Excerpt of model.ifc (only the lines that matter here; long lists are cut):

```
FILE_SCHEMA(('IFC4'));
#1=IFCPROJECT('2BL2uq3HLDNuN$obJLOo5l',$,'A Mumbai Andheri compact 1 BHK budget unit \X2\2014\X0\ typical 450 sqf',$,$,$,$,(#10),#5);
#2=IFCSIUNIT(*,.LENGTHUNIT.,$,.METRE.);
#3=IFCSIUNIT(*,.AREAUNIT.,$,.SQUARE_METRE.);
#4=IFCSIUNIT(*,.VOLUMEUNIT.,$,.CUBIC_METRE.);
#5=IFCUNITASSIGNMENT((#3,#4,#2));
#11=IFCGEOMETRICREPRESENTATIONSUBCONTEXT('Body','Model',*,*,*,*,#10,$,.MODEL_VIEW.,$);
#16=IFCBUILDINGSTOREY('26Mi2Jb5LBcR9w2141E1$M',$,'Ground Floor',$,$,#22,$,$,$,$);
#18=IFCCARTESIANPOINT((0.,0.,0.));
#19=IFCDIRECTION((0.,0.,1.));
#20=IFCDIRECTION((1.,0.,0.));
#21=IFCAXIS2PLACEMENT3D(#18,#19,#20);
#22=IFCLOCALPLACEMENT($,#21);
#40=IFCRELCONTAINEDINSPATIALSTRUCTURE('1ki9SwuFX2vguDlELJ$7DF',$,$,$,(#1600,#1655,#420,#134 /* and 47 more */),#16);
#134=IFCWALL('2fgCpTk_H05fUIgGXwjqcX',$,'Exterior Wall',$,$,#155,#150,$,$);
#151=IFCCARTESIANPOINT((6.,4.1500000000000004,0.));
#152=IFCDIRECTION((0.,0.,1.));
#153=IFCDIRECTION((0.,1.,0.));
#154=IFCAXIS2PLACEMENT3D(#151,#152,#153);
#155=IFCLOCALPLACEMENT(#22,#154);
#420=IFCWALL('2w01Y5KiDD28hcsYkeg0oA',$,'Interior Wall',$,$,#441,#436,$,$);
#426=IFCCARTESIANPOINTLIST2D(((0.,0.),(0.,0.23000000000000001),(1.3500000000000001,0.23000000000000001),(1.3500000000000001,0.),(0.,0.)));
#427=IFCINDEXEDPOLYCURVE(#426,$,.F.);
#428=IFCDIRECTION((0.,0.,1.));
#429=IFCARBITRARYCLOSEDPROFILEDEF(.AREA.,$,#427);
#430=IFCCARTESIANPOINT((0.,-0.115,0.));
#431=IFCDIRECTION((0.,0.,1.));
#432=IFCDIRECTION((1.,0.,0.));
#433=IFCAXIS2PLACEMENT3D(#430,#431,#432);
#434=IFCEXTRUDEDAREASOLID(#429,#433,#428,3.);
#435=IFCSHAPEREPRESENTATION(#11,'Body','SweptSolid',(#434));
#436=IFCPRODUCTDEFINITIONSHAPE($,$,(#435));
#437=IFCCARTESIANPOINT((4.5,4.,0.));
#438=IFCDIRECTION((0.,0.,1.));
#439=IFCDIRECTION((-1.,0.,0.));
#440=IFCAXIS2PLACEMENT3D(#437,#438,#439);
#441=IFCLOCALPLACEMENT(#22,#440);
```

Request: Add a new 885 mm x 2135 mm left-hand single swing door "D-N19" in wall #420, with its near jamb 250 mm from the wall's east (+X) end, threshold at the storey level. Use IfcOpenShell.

```python
import numpy as np
import ifcopenshell
import ifcopenshell.api.feature
import ifcopenshell.api.geometry
import ifcopenshell.api.root
import ifcopenshell.api.spatial
import ifcopenshell.geom
import ifcopenshell.util.element
import ifcopenshell.util.placement
import ifcopenshell.util.representation
import ifcopenshell.util.shape
import ifcopenshell.util.unit

model = ifcopenshell.open("model.ifc")
unit_scale = ifcopenshell.util.unit.calculate_unit_scale(model)
settings = ifcopenshell.geom.settings()


def volume(element):
    """Net volume in cubic metres, openings subtracted."""
    shape = ifcopenshell.geom.create_shape(settings, element)
    return ifcopenshell.util.shape.get_volume(shape.geometry)


wall = model.by_id(420)
storey = ifcopenshell.util.element.get_container(wall, ifc_class="IfcBuildingStorey")
context = ifcopenshell.util.representation.get_context(model, "Model", "Body", "MODEL_VIEW")
before = volume(wall)

width, height, from_end, sill = 0.885, 2.135, 0.25, 0.0  # metres

# The wall runs along its own X axis, and the end named is its -X end.
wall_shape = ifcopenshell.geom.create_shape(settings, wall)
x, y, z = ifcopenshell.util.shape.get_vertices(wall_shape.geometry).T
start = x.min() + from_end
face, thickness = float(y.min()), float(y.max() - y.min())
wall_matrix = ifcopenshell.util.placement.get_local_placement(wall.ObjectPlacement)
level = ifcopenshell.util.placement.get_local_placement(storey.ObjectPlacement)[2, 3]


def in_wall(x, y):
    """Placement at x, y metres in the wall's axes, at sill height."""
    matrix = wall_matrix.copy()
    matrix[:, 3] = wall_matrix @ np.array([x / unit_scale, y / unit_scale, 0.0, 1.0])
    matrix[2, 3] = level + sill / unit_scale
    return matrix


# Opening: a box that overshoots both wall faces by 50 mm.
opening = ifcopenshell.api.root.create_entity(model, ifc_class="IfcOpeningElement", predefined_type="OPENING")
box = ifcopenshell.api.geometry.add_wall_representation(
    model, context=context, length=width, height=height, thickness=thickness + 0.1
)
ifcopenshell.api.geometry.assign_representation(model, product=opening, representation=box)
ifcopenshell.api.geometry.edit_object_placement(model, product=opening, matrix=in_wall(start, face - 0.05), is_si=False)
ifcopenshell.api.feature.add_feature(model, feature=opening, element=wall)

door = ifcopenshell.api.root.create_entity(model, ifc_class="IfcDoor", name="D-N19", predefined_type="DOOR")
door.OverallWidth, door.OverallHeight = width / unit_scale, height / unit_scale
door.OperationType = "SINGLE_SWING_LEFT"
body = ifcopenshell.api.geometry.add_door_representation(
    model,
    context=context,
    overall_width=door.OverallWidth,
    overall_height=door.OverallHeight,
    operation_type="SINGLE_SWING_LEFT",
    lining_properties={"LiningDepth": thickness / unit_scale, "ThresholdDepth": thickness / unit_scale},
)
ifcopenshell.api.geometry.assign_representation(model, product=door, representation=body)
ifcopenshell.api.spatial.assign_container(model, products=[door], relating_structure=storey)
ifcopenshell.api.feature.add_filling(model, opening=opening, element=door)

# The lining spans the wall, so the door starts at the wall face.
ifcopenshell.api.geometry.edit_object_placement(model, product=door, matrix=in_wall(start, face), is_si=False)

after = volume(wall)

print(f"wall volume {before:.3f} -> {after:.3f} m3")

model.write("model_edited.ifc")
```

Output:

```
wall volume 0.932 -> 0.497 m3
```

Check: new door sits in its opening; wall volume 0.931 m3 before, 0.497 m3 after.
